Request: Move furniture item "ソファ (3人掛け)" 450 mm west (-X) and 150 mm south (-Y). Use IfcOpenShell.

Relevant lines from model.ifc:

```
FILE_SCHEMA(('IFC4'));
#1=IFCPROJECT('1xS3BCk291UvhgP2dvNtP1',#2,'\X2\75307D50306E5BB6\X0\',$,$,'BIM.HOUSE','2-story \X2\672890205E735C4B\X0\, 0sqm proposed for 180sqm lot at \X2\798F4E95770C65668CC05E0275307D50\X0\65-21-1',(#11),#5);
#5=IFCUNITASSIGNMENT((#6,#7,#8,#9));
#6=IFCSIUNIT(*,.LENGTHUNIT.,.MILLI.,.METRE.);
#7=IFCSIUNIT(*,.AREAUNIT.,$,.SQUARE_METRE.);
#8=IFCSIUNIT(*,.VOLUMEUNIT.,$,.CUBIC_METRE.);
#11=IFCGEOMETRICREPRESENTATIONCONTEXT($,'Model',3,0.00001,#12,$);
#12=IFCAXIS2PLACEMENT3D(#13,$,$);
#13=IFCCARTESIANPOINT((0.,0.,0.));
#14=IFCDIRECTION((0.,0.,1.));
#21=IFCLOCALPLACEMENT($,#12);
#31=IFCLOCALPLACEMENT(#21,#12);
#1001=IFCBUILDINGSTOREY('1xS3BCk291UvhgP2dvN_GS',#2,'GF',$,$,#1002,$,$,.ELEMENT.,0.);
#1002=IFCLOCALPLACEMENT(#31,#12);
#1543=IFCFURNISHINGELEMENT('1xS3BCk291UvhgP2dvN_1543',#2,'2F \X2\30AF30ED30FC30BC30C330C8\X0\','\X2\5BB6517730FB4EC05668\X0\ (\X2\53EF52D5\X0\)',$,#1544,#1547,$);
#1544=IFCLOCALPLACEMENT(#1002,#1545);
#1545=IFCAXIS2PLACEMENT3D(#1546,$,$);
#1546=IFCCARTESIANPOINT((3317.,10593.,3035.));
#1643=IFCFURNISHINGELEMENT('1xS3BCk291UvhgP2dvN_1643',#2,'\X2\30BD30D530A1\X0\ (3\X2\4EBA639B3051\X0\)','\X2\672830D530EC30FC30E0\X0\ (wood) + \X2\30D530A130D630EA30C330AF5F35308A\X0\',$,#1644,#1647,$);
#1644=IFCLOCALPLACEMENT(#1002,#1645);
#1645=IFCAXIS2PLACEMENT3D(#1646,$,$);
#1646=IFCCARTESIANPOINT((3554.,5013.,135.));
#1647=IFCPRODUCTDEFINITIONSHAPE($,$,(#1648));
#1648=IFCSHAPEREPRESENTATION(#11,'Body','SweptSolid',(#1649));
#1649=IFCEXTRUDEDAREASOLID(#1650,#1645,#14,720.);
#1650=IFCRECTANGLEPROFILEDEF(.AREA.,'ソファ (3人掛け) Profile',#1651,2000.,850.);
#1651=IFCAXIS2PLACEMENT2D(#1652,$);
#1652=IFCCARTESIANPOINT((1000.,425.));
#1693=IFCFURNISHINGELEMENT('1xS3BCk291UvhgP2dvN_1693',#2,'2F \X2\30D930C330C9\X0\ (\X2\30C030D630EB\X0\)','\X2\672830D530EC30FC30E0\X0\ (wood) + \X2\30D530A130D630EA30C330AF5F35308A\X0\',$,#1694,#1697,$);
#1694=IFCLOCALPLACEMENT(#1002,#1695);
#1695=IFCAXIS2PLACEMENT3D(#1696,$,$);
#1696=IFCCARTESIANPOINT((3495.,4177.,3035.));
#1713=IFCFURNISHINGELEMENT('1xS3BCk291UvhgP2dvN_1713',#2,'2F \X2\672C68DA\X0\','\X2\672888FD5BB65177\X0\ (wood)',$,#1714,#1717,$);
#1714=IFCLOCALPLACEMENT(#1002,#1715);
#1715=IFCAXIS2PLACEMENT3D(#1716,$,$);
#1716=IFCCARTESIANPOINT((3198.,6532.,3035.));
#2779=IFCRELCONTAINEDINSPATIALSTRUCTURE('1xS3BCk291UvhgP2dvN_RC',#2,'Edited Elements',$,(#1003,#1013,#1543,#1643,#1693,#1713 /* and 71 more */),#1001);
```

```python
import ifcopenshell
import ifcopenshell.api.geometry
import ifcopenshell.util.placement

model = ifcopenshell.open("model.ifc")

item = model.by_guid("1xS3BCk291UvhgP2dvN_1643")
matrix = ifcopenshell.util.placement.get_local_placement(item.ObjectPlacement)
matrix[0, 3] -= 450.0
matrix[1, 3] -= 150.0
ifcopenshell.api.geometry.edit_object_placement(model, product=item, matrix=matrix, is_si=False)

print(ifcopenshell.util.placement.get_local_placement(item.ObjectPlacement).round(3) + 0.0)

model.write("model_v2.ifc")
```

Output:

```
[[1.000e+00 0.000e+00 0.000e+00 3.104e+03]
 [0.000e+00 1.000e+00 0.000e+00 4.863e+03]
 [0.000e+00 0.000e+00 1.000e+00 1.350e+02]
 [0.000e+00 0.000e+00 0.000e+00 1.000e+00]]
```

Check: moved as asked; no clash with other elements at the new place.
